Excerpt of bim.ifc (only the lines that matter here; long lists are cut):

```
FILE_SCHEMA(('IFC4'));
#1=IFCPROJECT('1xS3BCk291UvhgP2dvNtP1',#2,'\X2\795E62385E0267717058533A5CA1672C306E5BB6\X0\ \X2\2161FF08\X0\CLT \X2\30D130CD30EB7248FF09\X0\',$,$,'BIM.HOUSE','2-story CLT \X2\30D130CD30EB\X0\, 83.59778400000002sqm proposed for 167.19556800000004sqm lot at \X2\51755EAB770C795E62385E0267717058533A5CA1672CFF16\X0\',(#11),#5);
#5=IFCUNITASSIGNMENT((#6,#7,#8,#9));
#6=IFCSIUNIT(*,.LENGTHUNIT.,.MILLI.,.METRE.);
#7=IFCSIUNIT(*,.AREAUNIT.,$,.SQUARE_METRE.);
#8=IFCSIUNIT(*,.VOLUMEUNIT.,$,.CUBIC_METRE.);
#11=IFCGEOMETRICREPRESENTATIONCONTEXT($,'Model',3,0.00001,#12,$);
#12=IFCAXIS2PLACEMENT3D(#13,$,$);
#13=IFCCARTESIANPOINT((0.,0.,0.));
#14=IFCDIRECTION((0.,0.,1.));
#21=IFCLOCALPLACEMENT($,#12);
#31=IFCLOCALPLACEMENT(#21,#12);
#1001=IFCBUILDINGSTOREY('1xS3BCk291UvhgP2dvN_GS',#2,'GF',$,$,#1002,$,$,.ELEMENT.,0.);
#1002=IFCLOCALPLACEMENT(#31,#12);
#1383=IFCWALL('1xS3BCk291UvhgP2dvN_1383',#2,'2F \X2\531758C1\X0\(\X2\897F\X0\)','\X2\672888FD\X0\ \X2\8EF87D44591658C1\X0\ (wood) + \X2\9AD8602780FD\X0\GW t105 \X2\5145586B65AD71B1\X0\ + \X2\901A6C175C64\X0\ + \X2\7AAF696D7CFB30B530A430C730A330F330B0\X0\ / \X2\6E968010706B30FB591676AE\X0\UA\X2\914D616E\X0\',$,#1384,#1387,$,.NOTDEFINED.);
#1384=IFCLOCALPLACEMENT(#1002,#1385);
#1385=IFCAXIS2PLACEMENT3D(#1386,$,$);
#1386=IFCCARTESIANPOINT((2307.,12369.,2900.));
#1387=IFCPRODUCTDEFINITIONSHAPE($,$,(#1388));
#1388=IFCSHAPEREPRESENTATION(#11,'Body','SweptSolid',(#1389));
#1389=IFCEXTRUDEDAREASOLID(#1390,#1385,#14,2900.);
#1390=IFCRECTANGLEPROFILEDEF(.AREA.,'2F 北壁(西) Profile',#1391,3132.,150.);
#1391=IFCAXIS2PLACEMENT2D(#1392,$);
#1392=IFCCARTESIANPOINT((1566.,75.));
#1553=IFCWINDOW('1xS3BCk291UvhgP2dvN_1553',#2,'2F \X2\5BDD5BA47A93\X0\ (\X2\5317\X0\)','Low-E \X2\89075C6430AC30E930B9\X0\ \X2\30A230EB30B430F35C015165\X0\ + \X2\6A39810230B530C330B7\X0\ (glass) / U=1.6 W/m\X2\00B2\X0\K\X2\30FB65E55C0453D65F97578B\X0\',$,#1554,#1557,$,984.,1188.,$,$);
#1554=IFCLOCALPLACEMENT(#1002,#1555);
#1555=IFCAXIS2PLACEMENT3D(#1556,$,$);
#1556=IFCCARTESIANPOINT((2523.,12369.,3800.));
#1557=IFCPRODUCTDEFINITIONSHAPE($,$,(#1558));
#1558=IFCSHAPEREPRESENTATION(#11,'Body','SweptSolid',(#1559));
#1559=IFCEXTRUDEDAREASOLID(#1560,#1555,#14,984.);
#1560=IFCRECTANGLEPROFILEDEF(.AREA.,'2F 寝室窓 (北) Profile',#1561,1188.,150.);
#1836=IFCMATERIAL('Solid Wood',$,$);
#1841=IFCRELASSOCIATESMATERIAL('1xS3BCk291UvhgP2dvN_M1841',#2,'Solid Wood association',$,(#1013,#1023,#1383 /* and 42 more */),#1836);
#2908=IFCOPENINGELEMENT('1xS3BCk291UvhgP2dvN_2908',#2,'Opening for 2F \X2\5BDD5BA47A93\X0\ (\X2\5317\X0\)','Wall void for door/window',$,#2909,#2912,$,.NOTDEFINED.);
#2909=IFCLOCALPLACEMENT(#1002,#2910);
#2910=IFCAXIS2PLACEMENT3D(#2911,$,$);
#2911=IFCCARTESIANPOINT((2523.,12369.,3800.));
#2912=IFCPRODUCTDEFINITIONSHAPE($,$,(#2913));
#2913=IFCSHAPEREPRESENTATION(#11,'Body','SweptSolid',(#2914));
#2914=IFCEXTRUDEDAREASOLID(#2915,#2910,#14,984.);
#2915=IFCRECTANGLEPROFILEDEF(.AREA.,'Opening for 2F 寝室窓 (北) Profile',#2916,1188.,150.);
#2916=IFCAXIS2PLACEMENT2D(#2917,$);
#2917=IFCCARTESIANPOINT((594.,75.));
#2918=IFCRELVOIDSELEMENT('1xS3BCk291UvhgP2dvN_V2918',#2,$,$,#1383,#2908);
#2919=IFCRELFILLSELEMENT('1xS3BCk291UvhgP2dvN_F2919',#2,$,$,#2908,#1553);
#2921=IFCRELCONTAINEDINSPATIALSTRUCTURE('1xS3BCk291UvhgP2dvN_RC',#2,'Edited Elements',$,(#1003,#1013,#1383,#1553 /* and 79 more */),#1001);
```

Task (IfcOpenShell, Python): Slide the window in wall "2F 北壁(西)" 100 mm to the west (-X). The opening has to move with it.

```python
import ifcopenshell
import ifcopenshell.api.geometry
import ifcopenshell.util.placement
import ifcopenshell.util.unit

model = ifcopenshell.open("bim.ifc")
unit_scale = ifcopenshell.util.unit.calculate_unit_scale(model)

window = model.by_guid("1xS3BCk291UvhgP2dvN_1553")
opening = window.FillsVoids[0].RelatingOpeningElement
wall = opening.VoidsElements[0].RelatingBuildingElement

wall_matrix = ifcopenshell.util.placement.get_local_placement(wall.ObjectPlacement)
shift = wall_matrix[:3, 0] * -0.1 / unit_scale
before = ifcopenshell.util.placement.get_local_placement(window.ObjectPlacement)[:3, 3].copy()

# The window is not placed relative to its opening, so move both.
for product in (opening, window):
    matrix = ifcopenshell.util.placement.get_local_placement(product.ObjectPlacement)
    matrix[:3, 3] += shift
    ifcopenshell.api.geometry.edit_object_placement(model, product=product, matrix=matrix, is_si=False)

after = ifcopenshell.util.placement.get_local_placement(window.ObjectPlacement)[:3, 3]
print("window moved by", (after - before).round(3) + 0.0)

model.write("bim_updated.ifc")
```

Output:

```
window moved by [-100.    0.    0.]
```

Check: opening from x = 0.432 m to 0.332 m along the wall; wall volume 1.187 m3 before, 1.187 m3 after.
